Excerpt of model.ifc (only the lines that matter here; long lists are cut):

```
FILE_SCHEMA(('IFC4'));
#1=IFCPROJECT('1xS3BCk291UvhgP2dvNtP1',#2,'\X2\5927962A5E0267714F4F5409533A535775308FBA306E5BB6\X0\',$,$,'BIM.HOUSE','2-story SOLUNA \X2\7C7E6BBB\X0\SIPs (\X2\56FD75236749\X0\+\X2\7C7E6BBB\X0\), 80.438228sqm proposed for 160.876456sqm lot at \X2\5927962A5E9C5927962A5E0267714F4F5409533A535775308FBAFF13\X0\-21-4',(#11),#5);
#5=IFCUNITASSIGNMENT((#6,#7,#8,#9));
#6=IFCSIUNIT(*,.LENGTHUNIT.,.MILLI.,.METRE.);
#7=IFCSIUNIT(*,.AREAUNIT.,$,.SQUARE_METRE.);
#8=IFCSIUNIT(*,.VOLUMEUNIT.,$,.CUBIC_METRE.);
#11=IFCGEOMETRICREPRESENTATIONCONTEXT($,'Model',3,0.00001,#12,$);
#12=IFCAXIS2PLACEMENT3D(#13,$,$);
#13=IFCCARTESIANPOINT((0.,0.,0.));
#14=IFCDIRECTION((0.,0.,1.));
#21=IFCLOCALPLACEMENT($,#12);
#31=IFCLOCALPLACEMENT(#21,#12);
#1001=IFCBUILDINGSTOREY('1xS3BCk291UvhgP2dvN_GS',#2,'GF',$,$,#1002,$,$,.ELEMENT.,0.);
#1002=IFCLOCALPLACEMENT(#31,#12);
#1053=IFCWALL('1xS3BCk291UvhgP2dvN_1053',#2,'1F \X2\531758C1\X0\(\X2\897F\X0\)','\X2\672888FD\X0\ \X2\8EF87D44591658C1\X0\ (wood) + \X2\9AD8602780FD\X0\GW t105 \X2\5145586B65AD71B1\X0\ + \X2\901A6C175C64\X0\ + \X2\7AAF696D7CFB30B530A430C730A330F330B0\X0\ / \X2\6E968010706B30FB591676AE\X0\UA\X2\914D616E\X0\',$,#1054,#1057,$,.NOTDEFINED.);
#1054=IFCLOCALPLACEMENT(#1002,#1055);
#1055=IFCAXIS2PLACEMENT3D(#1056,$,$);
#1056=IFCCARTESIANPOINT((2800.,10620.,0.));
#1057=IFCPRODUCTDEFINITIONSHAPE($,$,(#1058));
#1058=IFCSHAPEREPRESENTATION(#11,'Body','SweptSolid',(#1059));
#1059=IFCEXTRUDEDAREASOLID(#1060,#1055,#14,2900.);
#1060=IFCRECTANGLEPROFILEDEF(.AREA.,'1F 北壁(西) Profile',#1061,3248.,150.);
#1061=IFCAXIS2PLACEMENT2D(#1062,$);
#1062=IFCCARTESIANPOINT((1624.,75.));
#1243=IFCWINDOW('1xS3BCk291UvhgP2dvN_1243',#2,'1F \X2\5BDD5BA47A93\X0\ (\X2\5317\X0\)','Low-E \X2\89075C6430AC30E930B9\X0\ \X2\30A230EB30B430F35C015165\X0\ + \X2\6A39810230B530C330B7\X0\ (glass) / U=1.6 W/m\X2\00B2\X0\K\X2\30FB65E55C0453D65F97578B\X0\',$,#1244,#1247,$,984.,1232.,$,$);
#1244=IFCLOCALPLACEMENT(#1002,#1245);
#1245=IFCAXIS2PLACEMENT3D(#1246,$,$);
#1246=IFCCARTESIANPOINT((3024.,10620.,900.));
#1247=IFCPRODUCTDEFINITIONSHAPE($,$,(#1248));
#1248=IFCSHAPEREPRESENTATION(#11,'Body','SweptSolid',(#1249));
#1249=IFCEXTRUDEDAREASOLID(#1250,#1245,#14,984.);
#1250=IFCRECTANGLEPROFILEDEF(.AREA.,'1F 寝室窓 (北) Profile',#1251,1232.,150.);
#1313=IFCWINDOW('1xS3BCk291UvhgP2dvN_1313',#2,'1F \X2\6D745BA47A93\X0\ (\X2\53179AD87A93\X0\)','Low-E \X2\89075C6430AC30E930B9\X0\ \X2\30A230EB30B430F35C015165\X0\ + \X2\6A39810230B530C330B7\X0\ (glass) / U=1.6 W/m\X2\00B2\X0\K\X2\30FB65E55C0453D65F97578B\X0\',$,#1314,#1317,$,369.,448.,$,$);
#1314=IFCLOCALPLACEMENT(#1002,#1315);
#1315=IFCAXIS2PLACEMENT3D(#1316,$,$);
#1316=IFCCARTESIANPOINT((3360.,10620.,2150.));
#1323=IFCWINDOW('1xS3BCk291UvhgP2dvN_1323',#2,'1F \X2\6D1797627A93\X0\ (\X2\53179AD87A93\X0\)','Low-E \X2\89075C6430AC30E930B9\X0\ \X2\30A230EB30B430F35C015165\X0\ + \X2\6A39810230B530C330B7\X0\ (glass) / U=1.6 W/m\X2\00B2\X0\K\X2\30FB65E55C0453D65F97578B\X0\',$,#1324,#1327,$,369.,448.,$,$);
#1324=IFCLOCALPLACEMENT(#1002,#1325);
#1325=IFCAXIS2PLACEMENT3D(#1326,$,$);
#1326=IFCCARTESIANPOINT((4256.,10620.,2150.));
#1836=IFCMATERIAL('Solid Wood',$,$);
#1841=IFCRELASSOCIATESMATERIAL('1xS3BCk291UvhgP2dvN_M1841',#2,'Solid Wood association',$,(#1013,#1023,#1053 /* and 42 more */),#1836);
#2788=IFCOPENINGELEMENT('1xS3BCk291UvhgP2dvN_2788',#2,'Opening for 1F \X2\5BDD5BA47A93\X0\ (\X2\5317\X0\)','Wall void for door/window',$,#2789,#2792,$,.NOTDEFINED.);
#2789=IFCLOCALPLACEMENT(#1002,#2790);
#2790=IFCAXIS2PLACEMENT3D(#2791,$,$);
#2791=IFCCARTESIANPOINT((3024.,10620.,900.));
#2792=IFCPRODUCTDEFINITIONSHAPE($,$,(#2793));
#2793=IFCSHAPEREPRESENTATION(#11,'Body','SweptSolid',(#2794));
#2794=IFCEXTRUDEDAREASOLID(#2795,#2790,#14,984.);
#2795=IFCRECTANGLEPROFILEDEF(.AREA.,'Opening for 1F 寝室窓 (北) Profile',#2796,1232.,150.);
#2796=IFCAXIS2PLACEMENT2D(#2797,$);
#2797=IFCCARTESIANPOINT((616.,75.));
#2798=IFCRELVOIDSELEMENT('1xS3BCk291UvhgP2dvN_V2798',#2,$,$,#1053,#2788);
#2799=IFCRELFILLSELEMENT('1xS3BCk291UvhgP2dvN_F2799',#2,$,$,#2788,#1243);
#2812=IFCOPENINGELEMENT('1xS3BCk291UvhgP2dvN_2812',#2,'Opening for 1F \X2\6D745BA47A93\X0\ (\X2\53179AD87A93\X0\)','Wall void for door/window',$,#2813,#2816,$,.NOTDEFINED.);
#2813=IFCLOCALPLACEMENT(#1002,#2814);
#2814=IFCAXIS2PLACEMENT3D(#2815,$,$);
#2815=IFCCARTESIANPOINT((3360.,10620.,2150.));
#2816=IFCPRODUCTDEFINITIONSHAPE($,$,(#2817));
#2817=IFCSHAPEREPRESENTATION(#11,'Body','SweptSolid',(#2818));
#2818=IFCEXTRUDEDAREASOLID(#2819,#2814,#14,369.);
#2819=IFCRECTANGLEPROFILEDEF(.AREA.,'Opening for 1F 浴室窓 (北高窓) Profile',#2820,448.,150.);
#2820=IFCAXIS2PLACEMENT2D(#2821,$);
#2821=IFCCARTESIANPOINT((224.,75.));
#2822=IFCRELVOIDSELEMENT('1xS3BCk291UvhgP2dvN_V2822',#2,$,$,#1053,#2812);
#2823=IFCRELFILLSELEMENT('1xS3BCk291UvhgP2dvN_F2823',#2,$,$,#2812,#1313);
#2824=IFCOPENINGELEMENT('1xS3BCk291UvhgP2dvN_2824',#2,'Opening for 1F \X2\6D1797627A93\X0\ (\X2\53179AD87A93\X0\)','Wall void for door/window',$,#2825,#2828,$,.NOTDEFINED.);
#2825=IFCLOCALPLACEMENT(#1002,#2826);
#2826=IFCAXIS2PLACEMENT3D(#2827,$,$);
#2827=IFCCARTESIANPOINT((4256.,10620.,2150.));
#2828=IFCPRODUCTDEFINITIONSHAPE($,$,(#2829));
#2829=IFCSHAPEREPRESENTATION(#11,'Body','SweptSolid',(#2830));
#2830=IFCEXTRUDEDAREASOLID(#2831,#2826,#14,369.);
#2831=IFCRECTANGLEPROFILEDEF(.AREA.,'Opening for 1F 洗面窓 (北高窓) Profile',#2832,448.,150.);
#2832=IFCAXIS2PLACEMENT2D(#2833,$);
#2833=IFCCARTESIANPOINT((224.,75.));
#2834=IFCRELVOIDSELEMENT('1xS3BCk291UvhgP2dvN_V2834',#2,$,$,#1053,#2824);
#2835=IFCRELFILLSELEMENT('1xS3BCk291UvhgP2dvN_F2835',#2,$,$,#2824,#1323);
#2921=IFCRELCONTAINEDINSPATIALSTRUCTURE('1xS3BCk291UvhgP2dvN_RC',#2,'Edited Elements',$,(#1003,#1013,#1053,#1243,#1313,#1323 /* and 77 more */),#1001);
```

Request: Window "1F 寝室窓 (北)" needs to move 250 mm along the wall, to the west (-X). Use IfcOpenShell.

```python
import ifcopenshell
import ifcopenshell.api.geometry
import ifcopenshell.util.placement

model = ifcopenshell.open("model.ifc")

window = model.by_guid("1xS3BCk291UvhgP2dvN_1243")
opening = window.FillsVoids[0].RelatingOpeningElement
wall = opening.VoidsElements[0].RelatingBuildingElement

wall_matrix = ifcopenshell.util.placement.get_local_placement(wall.ObjectPlacement)
shift = wall_matrix[:3, 0] * -250.0
before = ifcopenshell.util.placement.get_local_placement(window.ObjectPlacement)[:3, 3].copy()

# The window is not placed relative to its opening, so move both.
for product in (opening, window):
    matrix = ifcopenshell.util.placement.get_local_placement(product.ObjectPlacement)
    matrix[:3, 3] += shift
    ifcopenshell.api.geometry.edit_object_placement(model, product=product, matrix=matrix, is_si=False)

after = ifcopenshell.util.placement.get_local_placement(window.ObjectPlacement)[:3, 3]
print("window moved by", (after - before).round(3) + 0.0)

model.write("model-out.ifc")
```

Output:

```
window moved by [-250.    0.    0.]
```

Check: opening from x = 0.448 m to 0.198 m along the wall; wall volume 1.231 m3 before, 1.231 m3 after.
